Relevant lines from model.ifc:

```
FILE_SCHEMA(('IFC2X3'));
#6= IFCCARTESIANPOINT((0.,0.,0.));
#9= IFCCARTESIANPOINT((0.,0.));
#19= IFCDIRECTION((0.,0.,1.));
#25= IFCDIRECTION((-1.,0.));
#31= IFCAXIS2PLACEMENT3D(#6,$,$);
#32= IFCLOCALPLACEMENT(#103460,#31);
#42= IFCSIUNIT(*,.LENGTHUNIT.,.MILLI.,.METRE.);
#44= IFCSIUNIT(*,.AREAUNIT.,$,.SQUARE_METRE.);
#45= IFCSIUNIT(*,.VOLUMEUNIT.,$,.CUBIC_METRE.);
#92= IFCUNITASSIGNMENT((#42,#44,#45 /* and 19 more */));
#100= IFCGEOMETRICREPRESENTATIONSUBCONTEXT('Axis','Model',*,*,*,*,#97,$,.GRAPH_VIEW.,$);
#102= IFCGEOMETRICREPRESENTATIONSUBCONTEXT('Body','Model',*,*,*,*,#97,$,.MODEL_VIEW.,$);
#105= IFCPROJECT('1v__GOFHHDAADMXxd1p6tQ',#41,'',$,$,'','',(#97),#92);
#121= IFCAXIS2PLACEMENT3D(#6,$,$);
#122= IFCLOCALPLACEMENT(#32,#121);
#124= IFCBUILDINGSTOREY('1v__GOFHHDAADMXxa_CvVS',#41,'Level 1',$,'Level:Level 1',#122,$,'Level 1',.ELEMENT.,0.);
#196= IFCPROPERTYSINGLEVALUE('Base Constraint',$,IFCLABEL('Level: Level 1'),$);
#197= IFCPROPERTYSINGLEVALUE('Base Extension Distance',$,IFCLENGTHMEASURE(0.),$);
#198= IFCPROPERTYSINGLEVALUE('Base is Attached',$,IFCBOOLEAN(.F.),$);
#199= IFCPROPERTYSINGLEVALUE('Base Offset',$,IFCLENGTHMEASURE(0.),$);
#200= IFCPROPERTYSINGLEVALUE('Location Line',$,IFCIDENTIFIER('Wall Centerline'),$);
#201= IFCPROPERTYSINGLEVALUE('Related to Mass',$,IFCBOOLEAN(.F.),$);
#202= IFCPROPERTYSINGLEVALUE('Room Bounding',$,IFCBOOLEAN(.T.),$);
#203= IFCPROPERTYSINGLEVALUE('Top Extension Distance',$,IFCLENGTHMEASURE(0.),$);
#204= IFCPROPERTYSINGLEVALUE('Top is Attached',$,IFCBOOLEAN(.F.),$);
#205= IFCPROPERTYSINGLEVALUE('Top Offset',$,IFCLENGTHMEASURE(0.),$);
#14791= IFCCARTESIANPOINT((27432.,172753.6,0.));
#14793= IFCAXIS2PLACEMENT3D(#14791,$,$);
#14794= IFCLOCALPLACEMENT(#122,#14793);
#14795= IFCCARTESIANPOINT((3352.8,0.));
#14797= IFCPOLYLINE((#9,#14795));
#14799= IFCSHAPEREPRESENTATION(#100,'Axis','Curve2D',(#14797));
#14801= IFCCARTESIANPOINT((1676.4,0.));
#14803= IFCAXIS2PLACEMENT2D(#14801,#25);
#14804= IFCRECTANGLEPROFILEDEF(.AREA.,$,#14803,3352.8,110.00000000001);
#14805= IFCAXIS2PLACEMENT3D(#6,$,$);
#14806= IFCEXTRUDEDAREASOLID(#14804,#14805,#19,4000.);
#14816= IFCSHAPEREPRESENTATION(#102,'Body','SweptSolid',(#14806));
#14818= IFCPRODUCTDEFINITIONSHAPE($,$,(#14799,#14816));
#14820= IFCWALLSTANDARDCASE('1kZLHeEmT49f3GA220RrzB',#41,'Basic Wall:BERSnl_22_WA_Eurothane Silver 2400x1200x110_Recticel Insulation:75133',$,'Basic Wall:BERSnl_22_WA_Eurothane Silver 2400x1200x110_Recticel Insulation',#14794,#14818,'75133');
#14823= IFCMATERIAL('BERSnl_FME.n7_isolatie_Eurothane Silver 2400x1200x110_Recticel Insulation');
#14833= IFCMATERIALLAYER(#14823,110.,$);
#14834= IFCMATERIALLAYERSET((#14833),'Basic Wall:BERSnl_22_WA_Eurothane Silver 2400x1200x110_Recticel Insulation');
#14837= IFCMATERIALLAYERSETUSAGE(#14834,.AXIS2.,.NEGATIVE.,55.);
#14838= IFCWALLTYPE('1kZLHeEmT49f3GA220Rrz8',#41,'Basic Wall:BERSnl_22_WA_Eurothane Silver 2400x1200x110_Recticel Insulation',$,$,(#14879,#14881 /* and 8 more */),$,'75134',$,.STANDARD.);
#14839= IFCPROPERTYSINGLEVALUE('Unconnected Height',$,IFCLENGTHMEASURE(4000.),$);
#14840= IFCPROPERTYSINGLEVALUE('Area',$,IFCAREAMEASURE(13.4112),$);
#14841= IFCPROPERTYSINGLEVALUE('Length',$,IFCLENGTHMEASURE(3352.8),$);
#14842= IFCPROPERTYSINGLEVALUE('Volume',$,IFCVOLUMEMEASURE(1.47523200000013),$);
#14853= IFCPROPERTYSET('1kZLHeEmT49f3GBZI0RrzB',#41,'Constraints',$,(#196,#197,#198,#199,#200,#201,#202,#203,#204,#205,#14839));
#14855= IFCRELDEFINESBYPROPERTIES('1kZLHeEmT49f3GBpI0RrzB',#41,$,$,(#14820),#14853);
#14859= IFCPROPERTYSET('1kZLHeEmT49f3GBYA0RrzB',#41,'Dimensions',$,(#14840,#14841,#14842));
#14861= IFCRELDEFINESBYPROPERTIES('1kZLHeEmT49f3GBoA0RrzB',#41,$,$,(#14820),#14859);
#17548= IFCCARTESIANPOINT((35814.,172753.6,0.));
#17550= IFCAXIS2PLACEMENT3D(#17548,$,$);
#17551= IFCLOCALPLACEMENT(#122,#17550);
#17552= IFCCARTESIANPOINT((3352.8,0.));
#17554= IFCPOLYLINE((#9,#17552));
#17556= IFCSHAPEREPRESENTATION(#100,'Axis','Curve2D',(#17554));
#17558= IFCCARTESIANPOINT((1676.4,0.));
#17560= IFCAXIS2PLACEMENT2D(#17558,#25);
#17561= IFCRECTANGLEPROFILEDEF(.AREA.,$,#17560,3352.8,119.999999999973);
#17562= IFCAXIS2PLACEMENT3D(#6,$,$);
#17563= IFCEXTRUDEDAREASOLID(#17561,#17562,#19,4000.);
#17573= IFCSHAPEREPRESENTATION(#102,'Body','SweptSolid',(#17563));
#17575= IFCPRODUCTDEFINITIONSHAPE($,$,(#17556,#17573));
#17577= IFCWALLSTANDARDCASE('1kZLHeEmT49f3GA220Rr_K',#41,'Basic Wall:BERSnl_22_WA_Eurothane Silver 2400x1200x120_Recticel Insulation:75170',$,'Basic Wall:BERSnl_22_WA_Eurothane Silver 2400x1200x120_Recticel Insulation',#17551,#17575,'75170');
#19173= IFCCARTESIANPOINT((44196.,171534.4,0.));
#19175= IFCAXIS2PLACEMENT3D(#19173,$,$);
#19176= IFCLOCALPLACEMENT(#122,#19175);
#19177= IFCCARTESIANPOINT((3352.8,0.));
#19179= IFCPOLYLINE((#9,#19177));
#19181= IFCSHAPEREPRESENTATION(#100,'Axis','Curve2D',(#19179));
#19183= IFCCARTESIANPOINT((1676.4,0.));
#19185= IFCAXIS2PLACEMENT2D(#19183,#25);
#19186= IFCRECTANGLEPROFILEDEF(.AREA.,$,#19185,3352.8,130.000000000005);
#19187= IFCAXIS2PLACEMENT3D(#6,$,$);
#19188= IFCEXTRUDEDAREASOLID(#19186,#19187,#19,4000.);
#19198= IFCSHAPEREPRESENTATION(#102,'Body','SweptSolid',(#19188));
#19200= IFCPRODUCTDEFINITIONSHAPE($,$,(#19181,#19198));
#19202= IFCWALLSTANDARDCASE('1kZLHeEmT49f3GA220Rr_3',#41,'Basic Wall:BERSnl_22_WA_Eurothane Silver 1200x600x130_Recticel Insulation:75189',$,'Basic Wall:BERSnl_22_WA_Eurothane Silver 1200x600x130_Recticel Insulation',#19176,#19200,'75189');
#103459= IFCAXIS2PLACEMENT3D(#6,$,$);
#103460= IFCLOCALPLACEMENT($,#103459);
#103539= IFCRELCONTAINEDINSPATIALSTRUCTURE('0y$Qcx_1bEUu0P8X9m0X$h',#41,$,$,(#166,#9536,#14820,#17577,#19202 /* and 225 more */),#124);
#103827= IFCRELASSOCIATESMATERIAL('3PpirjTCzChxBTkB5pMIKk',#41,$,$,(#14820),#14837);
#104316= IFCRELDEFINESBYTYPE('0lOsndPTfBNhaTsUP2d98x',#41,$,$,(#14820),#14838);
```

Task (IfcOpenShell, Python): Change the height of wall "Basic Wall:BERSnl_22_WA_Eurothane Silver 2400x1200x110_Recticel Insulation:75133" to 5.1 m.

```python
import ifcopenshell
import ifcopenshell.api.pset
import ifcopenshell.geom
import ifcopenshell.util.element
import ifcopenshell.util.representation
import ifcopenshell.util.shape
import ifcopenshell.util.unit

model = ifcopenshell.open("model.ifc")
unit_scale = ifcopenshell.util.unit.calculate_unit_scale(model)
area_scale = ifcopenshell.util.unit.calculate_unit_scale(model, "AREAUNIT")
volume_scale = ifcopenshell.util.unit.calculate_unit_scale(model, "VOLUMEUNIT")
settings = ifcopenshell.geom.settings()


def volume(element):
    """Net volume in cubic metres, openings subtracted."""
    shape = ifcopenshell.geom.create_shape(settings, element)
    return ifcopenshell.util.shape.get_volume(shape.geometry)


wall = model.by_guid("1kZLHeEmT49f3GA220RrzB")
before = volume(wall)

body = ifcopenshell.util.representation.get_representation(wall, "Model", "Body")
solid = body.Items[0]
old_height = solid.Depth
solid.Depth = 5.1 / unit_scale
after = volume(wall)
thickness = 0.11  # wall thickness in metres

# Update the stored height, areas and volumes.
pset = model.by_id(ifcopenshell.util.element.get_pset(wall, "Constraints", should_inherit=False)["id"])
ifcopenshell.api.pset.edit_pset(model, pset=pset, properties={
    "Unconnected Height": model.create_entity("IfcLengthMeasure", solid.Depth),
})
pset = model.by_id(ifcopenshell.util.element.get_pset(wall, "Dimensions", should_inherit=False)["id"])
ifcopenshell.api.pset.edit_pset(model, pset=pset, properties={
    "Area": model.create_entity("IfcAreaMeasure", after / thickness / area_scale),
    "Volume": model.create_entity("IfcVolumeMeasure", after / volume_scale),
})

print(f"height {old_height:g} -> {solid.Depth:g}, volume {before:.3f} -> {after:.3f} m3")

model.write("model_updated.ifc")
```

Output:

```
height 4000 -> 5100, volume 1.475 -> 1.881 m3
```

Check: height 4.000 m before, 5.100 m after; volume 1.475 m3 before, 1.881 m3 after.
